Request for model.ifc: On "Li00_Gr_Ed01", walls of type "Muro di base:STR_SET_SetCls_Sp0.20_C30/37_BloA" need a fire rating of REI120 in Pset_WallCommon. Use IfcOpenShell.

First a look at what the model holds.

```python
import ifcopenshell
import ifcopenshell.util.element

model = ifcopenshell.open("model.ifc")
print(model.schema)
storey = next(s for s in model.by_type("IfcBuildingStorey") if s.Name == "Li00_Gr_Ed01")
walls = [e for e in ifcopenshell.util.element.get_decomposition(storey) if e.is_a("IfcWall")]
seen = {}
for e in walls:
    element_type = ifcopenshell.util.element.get_type(e)
    key = (element_type.Name if element_type != e and element_type else None, ifcopenshell.util.element.get_pset(e, "Pset_WallCommon", "FireRating"))
    seen[key] = seen.get(key, 0) + 1
for (name, value), count in sorted(seen.items(), key=str):
    print(count, "x", name, "|", value)
```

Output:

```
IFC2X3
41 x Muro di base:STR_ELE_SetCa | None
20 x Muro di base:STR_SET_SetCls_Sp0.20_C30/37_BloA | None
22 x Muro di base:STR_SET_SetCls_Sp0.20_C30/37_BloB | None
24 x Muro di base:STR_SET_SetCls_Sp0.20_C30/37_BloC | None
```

```python
import ifcopenshell
import ifcopenshell.api.pset
import ifcopenshell.util.element

model = ifcopenshell.open("model.ifc")

storey = next(s for s in model.by_type("IfcBuildingStorey") if s.Name == "Li00_Gr_Ed01")
walls = [e for e in ifcopenshell.util.element.get_decomposition(storey) if e.is_a("IfcWall")]

count = 0
for e in walls:
    element_type = ifcopenshell.util.element.get_type(e)
    if element_type in (None, e) or element_type.Name != "Muro di base:STR_SET_SetCls_Sp0.20_C30/37_BloA":
        continue
    # add_pset returns the element's existing set when there is one.
    pset = ifcopenshell.api.pset.add_pset(model, product=e, name="Pset_WallCommon")
    ifcopenshell.api.pset.edit_pset(model, pset=pset, properties={"FireRating": "REI120"})
    count += 1

print(count, "walls updated")

model.write("model-out.ifc")
```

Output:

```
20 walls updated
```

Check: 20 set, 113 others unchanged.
